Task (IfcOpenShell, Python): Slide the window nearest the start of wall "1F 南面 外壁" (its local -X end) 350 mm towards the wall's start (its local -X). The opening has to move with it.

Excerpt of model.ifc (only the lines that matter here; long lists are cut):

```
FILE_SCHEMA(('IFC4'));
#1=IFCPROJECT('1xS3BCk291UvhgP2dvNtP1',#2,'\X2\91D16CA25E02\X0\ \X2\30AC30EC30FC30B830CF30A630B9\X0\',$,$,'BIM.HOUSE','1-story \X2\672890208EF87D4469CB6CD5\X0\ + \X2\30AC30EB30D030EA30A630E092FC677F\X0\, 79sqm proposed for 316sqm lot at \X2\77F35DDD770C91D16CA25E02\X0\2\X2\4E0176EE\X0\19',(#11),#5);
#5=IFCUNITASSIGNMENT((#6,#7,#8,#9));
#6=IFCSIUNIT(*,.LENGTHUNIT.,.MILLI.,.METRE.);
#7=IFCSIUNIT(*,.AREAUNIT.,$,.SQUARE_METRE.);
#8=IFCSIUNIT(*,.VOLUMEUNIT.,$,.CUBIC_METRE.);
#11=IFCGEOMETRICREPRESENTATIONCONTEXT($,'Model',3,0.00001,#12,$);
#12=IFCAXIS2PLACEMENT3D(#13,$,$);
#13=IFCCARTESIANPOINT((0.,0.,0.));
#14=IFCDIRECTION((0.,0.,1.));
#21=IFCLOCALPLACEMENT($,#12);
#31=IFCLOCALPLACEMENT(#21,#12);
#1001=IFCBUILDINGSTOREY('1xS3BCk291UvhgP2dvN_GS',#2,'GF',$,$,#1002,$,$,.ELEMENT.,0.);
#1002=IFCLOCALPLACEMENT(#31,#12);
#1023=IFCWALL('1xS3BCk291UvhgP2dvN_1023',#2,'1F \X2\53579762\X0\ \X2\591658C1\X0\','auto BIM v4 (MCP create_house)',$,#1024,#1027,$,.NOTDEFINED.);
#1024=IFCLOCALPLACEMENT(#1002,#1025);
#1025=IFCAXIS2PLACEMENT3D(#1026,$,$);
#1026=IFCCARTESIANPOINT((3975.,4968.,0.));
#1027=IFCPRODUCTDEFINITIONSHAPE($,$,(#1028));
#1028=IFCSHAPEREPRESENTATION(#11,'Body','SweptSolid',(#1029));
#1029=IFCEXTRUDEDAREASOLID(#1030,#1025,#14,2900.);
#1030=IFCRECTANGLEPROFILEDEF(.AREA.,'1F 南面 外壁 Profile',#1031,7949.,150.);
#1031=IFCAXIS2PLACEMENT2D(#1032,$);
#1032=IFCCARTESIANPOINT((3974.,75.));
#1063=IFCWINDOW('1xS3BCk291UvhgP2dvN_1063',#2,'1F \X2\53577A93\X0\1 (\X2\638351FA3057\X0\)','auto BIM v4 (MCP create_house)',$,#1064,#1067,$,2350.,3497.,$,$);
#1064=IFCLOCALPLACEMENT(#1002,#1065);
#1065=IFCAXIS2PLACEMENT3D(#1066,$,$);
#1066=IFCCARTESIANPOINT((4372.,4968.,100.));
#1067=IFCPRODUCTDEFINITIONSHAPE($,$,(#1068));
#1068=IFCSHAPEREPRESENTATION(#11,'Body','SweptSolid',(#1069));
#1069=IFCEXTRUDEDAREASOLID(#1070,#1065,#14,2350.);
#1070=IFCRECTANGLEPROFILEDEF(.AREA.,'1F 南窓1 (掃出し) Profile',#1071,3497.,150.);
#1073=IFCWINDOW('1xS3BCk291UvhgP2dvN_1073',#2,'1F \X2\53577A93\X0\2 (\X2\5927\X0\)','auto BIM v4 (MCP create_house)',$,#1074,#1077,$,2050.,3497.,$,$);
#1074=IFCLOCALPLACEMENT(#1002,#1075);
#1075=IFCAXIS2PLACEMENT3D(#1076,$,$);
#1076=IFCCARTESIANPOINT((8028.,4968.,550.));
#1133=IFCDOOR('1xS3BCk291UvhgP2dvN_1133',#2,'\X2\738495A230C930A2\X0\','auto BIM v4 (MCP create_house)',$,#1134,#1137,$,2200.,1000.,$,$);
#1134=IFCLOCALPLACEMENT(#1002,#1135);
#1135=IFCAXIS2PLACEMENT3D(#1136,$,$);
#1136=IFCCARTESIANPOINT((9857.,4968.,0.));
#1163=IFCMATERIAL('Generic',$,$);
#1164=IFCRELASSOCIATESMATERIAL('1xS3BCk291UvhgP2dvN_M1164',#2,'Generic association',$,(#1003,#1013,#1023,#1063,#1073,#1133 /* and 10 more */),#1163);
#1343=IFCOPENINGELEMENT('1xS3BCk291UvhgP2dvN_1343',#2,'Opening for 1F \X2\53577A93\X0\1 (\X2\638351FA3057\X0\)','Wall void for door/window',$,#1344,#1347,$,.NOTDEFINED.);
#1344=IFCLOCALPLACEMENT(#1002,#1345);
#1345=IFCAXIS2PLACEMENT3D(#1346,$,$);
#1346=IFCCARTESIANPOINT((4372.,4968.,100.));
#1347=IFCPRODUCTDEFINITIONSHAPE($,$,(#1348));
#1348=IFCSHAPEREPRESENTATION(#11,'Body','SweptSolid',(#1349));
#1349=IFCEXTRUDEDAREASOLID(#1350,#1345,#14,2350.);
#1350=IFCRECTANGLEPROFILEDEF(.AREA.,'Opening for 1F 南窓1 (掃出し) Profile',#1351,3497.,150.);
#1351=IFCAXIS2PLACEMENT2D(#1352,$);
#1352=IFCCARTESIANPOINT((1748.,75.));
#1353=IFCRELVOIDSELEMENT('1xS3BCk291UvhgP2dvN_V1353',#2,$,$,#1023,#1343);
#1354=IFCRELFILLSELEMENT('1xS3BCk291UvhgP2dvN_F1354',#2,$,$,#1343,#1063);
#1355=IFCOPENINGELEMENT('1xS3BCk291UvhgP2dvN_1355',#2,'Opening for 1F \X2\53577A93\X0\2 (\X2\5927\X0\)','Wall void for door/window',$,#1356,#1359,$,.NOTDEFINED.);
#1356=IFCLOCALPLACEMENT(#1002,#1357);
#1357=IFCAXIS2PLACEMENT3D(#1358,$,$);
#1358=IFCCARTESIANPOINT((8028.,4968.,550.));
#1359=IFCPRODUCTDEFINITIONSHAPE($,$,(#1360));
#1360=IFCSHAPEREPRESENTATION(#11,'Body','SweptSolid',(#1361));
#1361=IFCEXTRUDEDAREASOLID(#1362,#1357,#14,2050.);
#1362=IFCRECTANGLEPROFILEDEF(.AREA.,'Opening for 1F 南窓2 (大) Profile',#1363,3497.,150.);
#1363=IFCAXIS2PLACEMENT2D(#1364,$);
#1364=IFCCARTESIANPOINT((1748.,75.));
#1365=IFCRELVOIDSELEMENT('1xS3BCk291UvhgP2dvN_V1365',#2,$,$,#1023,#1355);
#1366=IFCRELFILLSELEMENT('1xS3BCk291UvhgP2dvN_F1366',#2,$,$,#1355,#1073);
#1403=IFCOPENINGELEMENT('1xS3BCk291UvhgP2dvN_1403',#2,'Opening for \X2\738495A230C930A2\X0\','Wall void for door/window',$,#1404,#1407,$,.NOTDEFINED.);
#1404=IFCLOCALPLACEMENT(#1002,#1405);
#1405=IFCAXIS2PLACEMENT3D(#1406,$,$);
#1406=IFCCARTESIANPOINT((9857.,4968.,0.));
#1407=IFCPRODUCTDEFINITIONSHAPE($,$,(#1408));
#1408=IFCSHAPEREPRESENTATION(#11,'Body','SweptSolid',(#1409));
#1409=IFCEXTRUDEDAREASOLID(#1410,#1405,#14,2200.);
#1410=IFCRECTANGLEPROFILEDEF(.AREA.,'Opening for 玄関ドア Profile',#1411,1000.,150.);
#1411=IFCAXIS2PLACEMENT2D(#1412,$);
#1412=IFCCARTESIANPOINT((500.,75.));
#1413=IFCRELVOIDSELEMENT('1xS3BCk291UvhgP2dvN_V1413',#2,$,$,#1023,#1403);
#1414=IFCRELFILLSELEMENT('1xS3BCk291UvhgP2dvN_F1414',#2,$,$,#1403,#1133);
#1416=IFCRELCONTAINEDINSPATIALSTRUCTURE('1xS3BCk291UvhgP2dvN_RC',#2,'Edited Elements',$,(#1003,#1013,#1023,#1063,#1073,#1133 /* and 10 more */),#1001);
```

```python
import ifcopenshell
import ifcopenshell.api.geometry
import ifcopenshell.util.placement

model = ifcopenshell.open("model.ifc")

window = model.by_id(1063)
opening = window.FillsVoids[0].RelatingOpeningElement
wall = opening.VoidsElements[0].RelatingBuildingElement

wall_matrix = ifcopenshell.util.placement.get_local_placement(wall.ObjectPlacement)
shift = wall_matrix[:3, 0] * -350.0
before = ifcopenshell.util.placement.get_local_placement(window.ObjectPlacement)[:3, 3].copy()

# The window is not placed relative to its opening, so move both.
for product in (opening, window):
    matrix = ifcopenshell.util.placement.get_local_placement(product.ObjectPlacement)
    matrix[:3, 3] += shift
    ifcopenshell.api.geometry.edit_object_placement(model, product=product, matrix=matrix, is_si=False)

after = ifcopenshell.util.placement.get_local_placement(window.ObjectPlacement)[:3, 3]
print("window moved by", (after - before).round(3) + 0.0)

model.write("model_v2.ifc")
```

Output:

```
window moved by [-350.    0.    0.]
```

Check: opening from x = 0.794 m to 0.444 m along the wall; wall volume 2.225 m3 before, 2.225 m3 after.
